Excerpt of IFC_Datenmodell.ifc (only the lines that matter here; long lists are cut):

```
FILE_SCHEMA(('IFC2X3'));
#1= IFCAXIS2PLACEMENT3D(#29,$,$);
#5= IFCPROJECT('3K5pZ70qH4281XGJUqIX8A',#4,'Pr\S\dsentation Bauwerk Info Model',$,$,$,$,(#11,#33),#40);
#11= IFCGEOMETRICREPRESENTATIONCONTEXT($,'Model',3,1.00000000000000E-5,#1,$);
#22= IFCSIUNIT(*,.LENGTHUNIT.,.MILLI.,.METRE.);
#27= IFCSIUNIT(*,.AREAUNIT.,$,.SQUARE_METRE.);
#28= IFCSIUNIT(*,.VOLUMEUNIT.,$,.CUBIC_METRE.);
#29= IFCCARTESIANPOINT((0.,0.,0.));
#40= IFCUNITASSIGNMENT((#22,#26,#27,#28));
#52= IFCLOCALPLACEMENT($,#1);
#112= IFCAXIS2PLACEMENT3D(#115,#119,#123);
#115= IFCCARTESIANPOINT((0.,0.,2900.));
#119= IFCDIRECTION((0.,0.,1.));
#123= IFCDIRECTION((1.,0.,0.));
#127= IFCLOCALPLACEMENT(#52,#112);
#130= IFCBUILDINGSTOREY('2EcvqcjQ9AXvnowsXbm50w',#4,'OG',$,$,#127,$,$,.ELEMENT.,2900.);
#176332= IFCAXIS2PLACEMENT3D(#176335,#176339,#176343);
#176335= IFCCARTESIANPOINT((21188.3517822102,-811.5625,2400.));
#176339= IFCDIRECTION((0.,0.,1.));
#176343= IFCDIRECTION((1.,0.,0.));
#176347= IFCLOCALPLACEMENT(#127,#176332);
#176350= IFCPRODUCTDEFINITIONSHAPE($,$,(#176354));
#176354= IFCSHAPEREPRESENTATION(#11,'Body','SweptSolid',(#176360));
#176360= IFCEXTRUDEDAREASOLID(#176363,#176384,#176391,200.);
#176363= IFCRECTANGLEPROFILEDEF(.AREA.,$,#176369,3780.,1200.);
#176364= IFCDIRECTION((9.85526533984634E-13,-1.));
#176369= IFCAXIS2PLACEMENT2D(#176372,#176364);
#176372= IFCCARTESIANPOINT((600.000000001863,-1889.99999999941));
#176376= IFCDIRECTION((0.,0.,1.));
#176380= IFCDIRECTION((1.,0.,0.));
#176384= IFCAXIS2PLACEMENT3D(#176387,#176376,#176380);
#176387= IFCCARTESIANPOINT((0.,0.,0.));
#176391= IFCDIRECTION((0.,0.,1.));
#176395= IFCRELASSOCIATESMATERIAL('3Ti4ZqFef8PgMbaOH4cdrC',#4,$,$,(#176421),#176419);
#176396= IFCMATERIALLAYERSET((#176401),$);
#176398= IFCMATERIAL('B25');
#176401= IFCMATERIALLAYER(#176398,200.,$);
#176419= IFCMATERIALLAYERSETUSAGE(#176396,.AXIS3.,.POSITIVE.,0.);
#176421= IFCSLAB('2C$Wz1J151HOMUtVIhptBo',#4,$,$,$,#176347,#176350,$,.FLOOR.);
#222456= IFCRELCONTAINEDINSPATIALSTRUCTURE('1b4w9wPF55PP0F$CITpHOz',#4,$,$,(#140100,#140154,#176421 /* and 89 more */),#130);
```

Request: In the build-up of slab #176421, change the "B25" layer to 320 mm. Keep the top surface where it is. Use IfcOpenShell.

```python
import ifcopenshell
import ifcopenshell.util.element
import ifcopenshell.util.unit

model = ifcopenshell.open("IFC_Datenmodell.ifc")
unit_scale = ifcopenshell.util.unit.calculate_unit_scale(model)

layer_set = model.by_id(176396)
layer = next(l for l in layer_set.MaterialLayers if l.Material and l.Material.Name == "B25")
change = 0.32 / unit_scale - layer.LayerThickness
layer.LayerThickness += change

# Geometry does not follow the layer set by itself.
slabs = [e for e in ifcopenshell.util.element.get_elements_by_material(model, layer_set) if e.is_a("IfcSlab")]
for slab in sorted(slabs, key=lambda e: e.id()):
    body = next(r for r in slab.Representation.Representations if r.RepresentationIdentifier == "Body")
    solid = body.Items[0]
    old_depth = solid.Depth
    solid.Depth += change
    # Extruded upwards: lower the start of the extrusion so the top stays.
    x, y, z = solid.Position.Location.Coordinates
    solid.Position.Location = model.createIfcCartesianPoint((x, y, z - change))
    print(slab.id(), f"{old_depth:g} -> {solid.Depth:g}")

# The layers are counted up from the underside, which has moved.
for usage in {ifcopenshell.util.element.get_material(slab) for slab in slabs}:
    usage.OffsetFromReferenceLine -= change

model.write("IFC_Datenmodell-out.ifc")
```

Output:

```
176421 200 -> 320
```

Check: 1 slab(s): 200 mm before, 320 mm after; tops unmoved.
